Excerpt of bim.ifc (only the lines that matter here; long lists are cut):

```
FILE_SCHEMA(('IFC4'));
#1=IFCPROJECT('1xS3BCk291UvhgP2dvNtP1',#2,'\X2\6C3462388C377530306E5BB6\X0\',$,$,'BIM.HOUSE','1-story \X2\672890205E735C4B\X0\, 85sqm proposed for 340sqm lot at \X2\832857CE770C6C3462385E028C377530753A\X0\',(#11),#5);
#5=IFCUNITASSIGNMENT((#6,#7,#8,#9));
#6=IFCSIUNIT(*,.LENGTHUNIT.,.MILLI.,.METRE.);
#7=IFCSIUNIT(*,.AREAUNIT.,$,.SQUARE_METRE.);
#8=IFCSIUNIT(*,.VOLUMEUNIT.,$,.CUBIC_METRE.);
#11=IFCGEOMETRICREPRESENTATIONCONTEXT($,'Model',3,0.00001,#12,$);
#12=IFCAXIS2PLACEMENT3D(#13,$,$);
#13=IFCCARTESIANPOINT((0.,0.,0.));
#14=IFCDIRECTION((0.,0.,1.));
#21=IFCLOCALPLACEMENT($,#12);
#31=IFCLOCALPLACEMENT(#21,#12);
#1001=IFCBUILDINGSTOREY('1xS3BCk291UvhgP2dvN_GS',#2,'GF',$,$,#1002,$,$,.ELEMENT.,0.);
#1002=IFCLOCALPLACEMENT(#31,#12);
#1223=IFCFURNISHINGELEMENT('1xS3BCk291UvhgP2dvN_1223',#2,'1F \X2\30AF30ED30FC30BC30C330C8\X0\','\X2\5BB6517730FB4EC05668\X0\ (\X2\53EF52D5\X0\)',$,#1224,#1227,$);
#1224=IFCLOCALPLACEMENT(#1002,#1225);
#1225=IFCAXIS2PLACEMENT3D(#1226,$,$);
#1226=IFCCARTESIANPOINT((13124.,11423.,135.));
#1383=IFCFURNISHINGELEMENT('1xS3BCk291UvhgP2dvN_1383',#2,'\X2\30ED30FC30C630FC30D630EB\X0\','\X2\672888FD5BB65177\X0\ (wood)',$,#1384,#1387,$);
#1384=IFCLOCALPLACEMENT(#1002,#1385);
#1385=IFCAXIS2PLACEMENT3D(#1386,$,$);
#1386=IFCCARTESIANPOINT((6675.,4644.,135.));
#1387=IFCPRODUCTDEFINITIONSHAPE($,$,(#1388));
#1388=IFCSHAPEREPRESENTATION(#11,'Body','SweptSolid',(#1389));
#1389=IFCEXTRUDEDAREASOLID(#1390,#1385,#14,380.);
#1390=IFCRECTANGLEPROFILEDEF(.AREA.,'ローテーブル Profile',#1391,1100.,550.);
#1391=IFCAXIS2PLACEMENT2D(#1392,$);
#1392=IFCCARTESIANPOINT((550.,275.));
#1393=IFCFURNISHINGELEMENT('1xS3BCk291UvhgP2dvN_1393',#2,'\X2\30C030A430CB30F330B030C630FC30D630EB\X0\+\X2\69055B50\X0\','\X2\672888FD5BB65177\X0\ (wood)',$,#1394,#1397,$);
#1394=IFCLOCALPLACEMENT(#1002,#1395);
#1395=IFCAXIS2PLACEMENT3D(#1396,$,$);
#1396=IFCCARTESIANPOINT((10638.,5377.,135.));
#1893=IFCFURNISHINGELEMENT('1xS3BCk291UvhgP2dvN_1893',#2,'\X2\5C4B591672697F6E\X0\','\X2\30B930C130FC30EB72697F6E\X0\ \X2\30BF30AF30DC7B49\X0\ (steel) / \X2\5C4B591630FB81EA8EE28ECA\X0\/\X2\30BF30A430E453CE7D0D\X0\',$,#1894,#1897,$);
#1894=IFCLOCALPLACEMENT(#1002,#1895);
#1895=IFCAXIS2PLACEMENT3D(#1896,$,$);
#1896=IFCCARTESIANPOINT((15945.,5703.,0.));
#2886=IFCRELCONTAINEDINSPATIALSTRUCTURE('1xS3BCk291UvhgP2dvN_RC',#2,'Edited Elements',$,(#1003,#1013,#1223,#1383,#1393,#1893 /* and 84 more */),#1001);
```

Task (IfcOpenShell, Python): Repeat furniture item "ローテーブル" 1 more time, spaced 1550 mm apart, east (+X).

```python
import numpy as np
import ifcopenshell
import ifcopenshell.api.geometry
import ifcopenshell.api.root
import ifcopenshell.util.element
import ifcopenshell.util.placement
import ifcopenshell.util.unit

model = ifcopenshell.open("bim.ifc")
unit_scale = ifcopenshell.util.unit.calculate_unit_scale(model)


def reuse_history(source, copy):
    """copy_class also copies each property set's owner history, people and application; keep the originals."""
    for rel in copy.IsDefinedBy:
        if rel.is_a("IfcRelDefinesByProperties") and (history := rel.RelatingPropertyDefinition.OwnerHistory):
            rel.RelatingPropertyDefinition.OwnerHistory = source.OwnerHistory
            ifcopenshell.util.element.remove_deep2(model, history)


source = model.by_guid("1xS3BCk291UvhgP2dvN_1383")
base = ifcopenshell.util.placement.get_local_placement(source.ObjectPlacement)
step = np.array([1.0, 0.0, 0.0]) * 1.55 / unit_scale

for i in range(1, 2):
    copy = ifcopenshell.api.root.copy_class(model, product=source)
    copy.Representation = ifcopenshell.util.element.copy_deep(
        model, source.Representation, exclude=["IfcGeometricRepresentationContext", "IfcRepresentationMap"]
    )
    reuse_history(source, copy)
    matrix = base.copy()
    matrix[:3, 3] += i * step
    print("added at", matrix[:3, 3].round(3) + 0.0)
    ifcopenshell.api.geometry.edit_object_placement(model, product=copy, matrix=matrix, is_si=False)

model.write("bim-out.ifc")
```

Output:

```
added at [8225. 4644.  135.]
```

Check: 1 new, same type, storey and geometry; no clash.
